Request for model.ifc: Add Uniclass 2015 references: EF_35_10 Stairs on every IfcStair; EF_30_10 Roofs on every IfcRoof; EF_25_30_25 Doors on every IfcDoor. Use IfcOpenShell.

First a look at what the model holds.

```python
import ifcopenshell

model = ifcopenshell.open("model.ifc")
print(model.schema)
print("classifications:", [c.Name for c in model.by_type("IfcClassification")])
for ifc_class in ("IfcDoor", "IfcRoof", "IfcStair", "IfcWall", "IfcWindow"):
    print(ifc_class, len(model.by_type(ifc_class)))
```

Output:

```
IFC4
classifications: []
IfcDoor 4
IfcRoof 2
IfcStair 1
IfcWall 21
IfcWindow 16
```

```python
import ifcopenshell
import ifcopenshell.api.classification

model = ifcopenshell.open("model.ifc")

system = ifcopenshell.api.classification.add_classification(model, classification="Uniclass 2015")

codes = {
    "IfcStair": ("EF_35_10", "Stairs"),
    "IfcRoof": ("EF_30_10", "Roofs"),
    "IfcDoor": ("EF_25_30_25", "Doors"),
}
for ifc_class, (code, name) in codes.items():
    products = model.by_type(ifc_class)
    ifcopenshell.api.classification.add_reference(
        model, products=products, classification=system, identification=code, name=name
    )
    print(code, len(products))

model.write("model-out.ifc")
```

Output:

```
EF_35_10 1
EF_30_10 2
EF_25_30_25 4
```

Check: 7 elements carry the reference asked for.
